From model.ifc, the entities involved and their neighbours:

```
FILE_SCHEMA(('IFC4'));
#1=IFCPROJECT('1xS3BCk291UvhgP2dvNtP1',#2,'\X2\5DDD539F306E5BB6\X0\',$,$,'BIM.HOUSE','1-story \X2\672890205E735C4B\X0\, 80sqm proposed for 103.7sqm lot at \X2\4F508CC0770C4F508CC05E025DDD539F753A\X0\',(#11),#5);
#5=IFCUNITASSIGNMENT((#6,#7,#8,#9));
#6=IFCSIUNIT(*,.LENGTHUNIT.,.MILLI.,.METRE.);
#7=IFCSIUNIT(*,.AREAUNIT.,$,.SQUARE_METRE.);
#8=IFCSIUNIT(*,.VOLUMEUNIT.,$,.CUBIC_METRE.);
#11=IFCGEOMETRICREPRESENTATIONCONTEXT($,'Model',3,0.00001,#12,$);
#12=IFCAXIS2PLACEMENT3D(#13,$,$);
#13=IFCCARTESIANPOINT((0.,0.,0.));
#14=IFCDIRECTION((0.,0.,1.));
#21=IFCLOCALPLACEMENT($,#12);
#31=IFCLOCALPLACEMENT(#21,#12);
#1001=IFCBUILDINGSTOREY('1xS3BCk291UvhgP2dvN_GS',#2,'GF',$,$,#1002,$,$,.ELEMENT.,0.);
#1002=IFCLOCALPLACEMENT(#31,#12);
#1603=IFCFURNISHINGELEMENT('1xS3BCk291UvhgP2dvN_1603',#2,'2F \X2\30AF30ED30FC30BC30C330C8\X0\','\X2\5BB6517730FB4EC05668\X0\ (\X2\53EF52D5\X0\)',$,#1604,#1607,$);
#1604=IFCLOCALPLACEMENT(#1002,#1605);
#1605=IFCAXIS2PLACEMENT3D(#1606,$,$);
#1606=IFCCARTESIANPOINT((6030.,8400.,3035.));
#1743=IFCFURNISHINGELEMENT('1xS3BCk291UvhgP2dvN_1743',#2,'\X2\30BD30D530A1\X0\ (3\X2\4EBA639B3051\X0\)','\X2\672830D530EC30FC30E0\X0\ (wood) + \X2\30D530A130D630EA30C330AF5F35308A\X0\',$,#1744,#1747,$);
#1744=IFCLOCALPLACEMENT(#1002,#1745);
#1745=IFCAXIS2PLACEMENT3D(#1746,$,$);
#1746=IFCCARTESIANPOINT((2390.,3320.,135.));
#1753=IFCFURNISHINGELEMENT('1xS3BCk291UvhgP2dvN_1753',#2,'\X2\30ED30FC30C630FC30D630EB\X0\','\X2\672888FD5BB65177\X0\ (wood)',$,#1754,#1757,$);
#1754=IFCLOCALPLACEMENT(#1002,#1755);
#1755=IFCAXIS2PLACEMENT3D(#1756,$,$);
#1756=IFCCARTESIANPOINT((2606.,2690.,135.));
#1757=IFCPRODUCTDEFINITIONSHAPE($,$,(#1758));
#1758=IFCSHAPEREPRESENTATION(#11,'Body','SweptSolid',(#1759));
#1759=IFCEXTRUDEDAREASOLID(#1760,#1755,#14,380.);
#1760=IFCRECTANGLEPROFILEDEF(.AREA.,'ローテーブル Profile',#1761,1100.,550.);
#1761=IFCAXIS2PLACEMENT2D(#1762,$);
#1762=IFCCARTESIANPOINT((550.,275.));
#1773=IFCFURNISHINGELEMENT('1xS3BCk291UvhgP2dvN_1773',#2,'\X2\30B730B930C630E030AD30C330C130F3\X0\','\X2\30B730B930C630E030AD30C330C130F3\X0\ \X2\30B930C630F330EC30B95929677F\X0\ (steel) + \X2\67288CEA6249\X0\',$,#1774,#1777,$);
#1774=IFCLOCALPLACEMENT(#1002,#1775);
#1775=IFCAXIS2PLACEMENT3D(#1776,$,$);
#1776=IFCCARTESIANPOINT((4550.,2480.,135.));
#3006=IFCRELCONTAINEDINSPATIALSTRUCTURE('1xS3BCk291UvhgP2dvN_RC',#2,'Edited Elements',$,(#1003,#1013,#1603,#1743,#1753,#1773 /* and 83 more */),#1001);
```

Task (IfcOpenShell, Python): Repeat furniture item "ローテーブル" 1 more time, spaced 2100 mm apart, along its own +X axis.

```python
import ifcopenshell
import ifcopenshell.api.geometry
import ifcopenshell.api.root
import ifcopenshell.util.element
import ifcopenshell.util.placement

model = ifcopenshell.open("model.ifc")


def reuse_history(source, copy):
    """copy_class also copies each property set's owner history, people and application; keep the originals."""
    for rel in copy.IsDefinedBy:
        if rel.is_a("IfcRelDefinesByProperties") and (history := rel.RelatingPropertyDefinition.OwnerHistory):
            rel.RelatingPropertyDefinition.OwnerHistory = source.OwnerHistory
            ifcopenshell.util.element.remove_deep2(model, history)


source = model.by_id(1753)
base = ifcopenshell.util.placement.get_local_placement(source.ObjectPlacement)
step = base[:3, 0] * 2100.0

for i in range(1, 2):
    copy = ifcopenshell.api.root.copy_class(model, product=source)
    copy.Representation = ifcopenshell.util.element.copy_deep(
        model, source.Representation, exclude=["IfcGeometricRepresentationContext", "IfcRepresentationMap"]
    )
    reuse_history(source, copy)
    matrix = base.copy()
    matrix[:3, 3] += i * step
    print("added at", matrix[:3, 3].round(3) + 0.0)
    ifcopenshell.api.geometry.edit_object_placement(model, product=copy, matrix=matrix, is_si=False)

model.write("model_v2.ifc")
```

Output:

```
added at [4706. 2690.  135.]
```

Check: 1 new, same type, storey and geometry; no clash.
